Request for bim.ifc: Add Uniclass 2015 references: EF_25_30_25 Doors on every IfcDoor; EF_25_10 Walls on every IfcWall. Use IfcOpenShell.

First a look at what the model holds.

```python
import ifcopenshell

model = ifcopenshell.open("bim.ifc")
print(model.schema)
print("classifications:", [c.Name for c in model.by_type("IfcClassification")])
for ifc_class in ("IfcDoor", "IfcRoof", "IfcStair", "IfcWall", "IfcWindow"):
    print(ifc_class, len(model.by_type(ifc_class)))
```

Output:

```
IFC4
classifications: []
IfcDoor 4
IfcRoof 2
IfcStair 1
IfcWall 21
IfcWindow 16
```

```python
import ifcopenshell
import ifcopenshell.api.classification

model = ifcopenshell.open("bim.ifc")

system = ifcopenshell.api.classification.add_classification(model, classification="Uniclass 2015")

codes = {
    "IfcDoor": ("EF_25_30_25", "Doors"),
    "IfcWall": ("EF_25_10", "Walls"),
}
for ifc_class, (code, name) in codes.items():
    products = model.by_type(ifc_class)
    ifcopenshell.api.classification.add_reference(
        model, products=products, classification=system, identification=code, name=name
    )
    print(code, len(products))

model.write("bim_v2.ifc")
```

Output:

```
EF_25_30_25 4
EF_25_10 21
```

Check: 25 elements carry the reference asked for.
